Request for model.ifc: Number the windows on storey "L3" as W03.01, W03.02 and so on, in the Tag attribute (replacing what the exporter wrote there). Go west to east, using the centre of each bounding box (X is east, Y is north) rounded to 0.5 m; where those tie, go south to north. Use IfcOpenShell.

First a look at what the model holds.

```python
import ifcopenshell
import ifcopenshell.util.element
import ifcopenshell.util.placement

model = ifcopenshell.open("model.ifc")
print(model.schema)
storey = next(s for s in model.by_type("IfcBuildingStorey") if s.Name == "L3")
windows = [e for e in ifcopenshell.util.element.get_decomposition(storey) if e.is_a("IfcWindow")]
for e in sorted(windows, key=lambda e: e.id()):
    origin = ifcopenshell.util.placement.get_local_placement(e.ObjectPlacement)[:3, 3]
    print(e.id(), e.Tag, e.Name, origin.round(2) + 0.0, sep=" | ")
```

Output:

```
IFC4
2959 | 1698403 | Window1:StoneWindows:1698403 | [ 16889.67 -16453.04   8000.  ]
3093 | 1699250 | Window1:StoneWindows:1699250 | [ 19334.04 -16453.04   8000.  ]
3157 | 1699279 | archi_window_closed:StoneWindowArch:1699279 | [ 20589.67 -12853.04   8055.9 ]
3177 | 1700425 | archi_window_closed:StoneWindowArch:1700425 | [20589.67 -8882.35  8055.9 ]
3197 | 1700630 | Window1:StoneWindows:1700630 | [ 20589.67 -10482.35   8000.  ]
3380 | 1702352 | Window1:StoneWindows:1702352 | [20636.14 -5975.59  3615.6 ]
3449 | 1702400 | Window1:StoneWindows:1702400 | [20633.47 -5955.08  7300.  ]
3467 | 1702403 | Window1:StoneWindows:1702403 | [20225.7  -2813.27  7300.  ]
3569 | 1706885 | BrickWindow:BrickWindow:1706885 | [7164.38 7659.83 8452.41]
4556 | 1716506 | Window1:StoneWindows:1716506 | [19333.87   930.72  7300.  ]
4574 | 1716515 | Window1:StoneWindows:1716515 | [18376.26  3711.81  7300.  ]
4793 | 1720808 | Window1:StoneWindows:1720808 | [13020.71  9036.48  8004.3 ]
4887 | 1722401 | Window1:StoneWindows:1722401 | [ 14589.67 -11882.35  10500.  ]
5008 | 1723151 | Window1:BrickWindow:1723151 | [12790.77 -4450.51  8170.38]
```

```python
import ifcopenshell
import ifcopenshell.geom
import ifcopenshell.util.element
import ifcopenshell.util.shape

model = ifcopenshell.open("model.ifc")
settings = ifcopenshell.geom.settings()
settings.set("use-world-coords", True)


def centre(element):
    shape = ifcopenshell.geom.create_shape(settings, element)
    return ifcopenshell.util.shape.get_bbox_centroid(shape.geometry)


storey = next(s for s in model.by_type("IfcBuildingStorey") if s.Name == "L3")
windows = [e for e in ifcopenshell.util.element.get_decomposition(storey) if e.is_a("IfcWindow")]

# Insertion points can sit at a corner or the storey origin, so sort by the geometry (in metres).
centres = {e: centre(e) for e in windows}
windows.sort(key=lambda e: (round(centres[e][0] / 0.5), centres[e][1]))

for i, e in enumerate(windows, start=1):
    number = f"W03.{i:02d}"
    e.Tag = number
    print(e.id(), number)

model.write("model_rev.ifc")
```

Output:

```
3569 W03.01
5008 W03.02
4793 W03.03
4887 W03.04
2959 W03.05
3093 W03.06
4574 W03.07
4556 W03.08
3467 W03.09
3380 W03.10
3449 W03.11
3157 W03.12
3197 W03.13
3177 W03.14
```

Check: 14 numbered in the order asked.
